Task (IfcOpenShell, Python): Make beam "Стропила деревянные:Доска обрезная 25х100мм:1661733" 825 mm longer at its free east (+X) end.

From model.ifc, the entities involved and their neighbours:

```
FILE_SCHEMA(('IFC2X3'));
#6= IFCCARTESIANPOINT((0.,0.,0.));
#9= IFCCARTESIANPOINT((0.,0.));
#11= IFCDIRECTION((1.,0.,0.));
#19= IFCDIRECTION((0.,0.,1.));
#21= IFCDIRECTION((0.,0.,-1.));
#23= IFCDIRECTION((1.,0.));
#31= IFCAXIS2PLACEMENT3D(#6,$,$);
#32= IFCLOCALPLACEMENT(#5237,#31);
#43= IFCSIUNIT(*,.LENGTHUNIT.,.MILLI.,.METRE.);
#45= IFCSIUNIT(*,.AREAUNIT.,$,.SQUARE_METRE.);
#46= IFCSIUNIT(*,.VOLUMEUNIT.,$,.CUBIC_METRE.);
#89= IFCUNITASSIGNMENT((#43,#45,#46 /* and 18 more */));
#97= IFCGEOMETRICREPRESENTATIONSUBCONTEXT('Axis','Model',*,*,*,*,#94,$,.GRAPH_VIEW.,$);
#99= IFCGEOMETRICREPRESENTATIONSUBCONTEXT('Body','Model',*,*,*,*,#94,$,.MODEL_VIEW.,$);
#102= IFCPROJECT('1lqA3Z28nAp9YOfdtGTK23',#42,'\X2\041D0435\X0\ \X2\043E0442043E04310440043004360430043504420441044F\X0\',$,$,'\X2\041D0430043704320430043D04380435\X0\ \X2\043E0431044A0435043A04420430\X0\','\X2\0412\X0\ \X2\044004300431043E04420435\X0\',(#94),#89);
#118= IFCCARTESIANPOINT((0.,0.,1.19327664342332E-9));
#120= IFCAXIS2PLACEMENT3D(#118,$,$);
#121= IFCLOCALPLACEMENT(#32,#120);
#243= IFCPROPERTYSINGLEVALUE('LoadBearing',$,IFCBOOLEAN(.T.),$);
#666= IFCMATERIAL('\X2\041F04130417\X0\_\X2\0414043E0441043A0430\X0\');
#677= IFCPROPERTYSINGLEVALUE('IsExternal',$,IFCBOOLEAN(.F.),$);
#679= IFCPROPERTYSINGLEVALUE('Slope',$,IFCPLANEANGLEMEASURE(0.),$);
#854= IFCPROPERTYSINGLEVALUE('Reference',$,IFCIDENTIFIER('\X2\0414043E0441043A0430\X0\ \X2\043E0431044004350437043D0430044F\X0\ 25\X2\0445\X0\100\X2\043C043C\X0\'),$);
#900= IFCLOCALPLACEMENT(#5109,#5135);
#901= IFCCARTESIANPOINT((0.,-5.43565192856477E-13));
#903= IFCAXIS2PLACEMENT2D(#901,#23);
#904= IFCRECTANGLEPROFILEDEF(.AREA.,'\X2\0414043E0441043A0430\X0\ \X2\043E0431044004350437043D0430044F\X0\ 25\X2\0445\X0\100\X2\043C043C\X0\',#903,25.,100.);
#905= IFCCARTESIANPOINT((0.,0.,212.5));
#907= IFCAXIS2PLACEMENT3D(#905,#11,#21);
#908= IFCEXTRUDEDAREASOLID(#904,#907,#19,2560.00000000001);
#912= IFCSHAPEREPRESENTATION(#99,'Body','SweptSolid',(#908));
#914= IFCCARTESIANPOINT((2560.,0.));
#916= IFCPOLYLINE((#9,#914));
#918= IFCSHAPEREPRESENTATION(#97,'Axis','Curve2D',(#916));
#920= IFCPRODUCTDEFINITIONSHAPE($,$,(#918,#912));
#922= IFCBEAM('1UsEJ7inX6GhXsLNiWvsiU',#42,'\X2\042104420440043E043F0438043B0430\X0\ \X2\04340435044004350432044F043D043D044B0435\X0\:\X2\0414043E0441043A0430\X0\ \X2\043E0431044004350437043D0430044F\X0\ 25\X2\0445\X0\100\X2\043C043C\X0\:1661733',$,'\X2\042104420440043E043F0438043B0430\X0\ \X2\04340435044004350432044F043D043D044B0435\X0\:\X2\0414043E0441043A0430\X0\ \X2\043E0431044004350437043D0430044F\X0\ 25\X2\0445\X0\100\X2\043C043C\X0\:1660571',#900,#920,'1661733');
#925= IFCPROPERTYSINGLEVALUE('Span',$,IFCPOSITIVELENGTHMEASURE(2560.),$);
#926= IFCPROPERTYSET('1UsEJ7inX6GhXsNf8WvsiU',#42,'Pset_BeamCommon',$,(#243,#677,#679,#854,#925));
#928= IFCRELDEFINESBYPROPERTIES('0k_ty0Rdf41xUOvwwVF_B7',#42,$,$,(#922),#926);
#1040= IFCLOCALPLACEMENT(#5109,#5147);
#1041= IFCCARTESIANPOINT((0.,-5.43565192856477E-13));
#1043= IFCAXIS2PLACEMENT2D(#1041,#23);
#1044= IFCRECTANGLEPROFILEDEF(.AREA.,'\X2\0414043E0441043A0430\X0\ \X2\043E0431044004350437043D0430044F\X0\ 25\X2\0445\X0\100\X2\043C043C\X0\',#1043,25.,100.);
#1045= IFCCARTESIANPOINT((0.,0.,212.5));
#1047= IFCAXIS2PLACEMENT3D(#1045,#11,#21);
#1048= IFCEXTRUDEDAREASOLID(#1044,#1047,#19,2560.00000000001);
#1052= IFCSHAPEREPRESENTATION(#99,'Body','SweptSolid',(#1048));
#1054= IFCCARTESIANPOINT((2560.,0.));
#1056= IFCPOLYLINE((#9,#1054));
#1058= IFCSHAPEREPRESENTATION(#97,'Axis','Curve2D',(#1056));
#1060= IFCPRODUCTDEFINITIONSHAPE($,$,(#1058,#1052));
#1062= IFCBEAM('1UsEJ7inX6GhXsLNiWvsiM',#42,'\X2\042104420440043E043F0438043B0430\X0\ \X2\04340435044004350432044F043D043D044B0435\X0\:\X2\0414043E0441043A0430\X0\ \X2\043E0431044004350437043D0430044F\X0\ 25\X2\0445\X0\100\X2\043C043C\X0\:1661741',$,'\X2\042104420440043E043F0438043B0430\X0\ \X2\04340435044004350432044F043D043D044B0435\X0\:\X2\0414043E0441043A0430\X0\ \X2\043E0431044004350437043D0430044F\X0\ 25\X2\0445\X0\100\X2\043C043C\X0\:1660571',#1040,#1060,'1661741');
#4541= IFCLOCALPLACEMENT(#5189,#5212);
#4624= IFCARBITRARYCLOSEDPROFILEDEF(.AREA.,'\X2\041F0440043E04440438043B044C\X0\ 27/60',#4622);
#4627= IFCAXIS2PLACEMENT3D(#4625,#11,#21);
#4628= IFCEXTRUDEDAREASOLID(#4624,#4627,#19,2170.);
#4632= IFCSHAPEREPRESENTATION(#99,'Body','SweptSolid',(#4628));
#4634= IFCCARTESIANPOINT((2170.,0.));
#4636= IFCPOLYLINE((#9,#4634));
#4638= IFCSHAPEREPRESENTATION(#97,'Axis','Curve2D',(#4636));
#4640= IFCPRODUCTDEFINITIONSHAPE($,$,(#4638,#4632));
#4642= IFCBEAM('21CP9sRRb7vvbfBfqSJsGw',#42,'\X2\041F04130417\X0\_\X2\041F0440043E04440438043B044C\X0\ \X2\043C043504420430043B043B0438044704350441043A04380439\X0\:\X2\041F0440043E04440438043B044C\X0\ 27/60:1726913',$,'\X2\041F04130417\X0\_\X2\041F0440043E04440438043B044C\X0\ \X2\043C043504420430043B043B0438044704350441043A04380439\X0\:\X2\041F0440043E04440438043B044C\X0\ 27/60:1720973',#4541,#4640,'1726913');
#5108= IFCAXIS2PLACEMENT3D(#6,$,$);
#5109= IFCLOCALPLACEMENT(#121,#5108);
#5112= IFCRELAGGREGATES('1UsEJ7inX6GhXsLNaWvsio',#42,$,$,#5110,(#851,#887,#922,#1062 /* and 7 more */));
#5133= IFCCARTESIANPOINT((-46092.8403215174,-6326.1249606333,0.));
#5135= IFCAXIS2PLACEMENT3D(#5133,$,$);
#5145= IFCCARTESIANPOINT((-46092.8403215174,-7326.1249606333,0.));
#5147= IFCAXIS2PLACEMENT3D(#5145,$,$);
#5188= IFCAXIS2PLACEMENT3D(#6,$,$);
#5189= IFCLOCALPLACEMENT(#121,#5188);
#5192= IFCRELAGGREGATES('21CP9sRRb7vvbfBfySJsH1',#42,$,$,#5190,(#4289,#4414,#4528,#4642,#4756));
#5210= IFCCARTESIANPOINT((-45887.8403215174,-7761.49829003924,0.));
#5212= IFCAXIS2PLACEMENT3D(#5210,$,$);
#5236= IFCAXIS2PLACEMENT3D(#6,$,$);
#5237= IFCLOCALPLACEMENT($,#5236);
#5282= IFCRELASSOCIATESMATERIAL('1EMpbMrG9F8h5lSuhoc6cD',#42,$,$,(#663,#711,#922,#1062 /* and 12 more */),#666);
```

```python
import numpy as np
import ifcopenshell
import ifcopenshell.api.pset
import ifcopenshell.util.element
import ifcopenshell.util.representation
import ifcopenshell.util.unit

model = ifcopenshell.open("model.ifc")
unit_scale = ifcopenshell.util.unit.calculate_unit_scale(model)

member = model.by_guid("1UsEJ7inX6GhXsLNiWvsiU")
change = 0.825 / unit_scale

# The extrusion runs towards the end named, so only its depth changes.
body = ifcopenshell.util.representation.get_representation(member, "Model", "Body")
solid = body.Items[0]
old_length = solid.Depth
solid.Depth += change

# Move the axis end point with it.
axis = next(r for r in member.Representation.Representations if r.RepresentationIdentifier == "Axis").Items[0]
start, end = (np.array(p.Coordinates) for p in axis.Points)
end = end + (end - start) / np.linalg.norm(end - start) * change
point = model.createIfcCartesianPoint(end.tolist())
axis.Points = [axis.Points[0], point]

# Update the stored length and volume.
pset = model.by_id(ifcopenshell.util.element.get_pset(member, "Pset_BeamCommon", should_inherit=False)["id"])
ifcopenshell.api.pset.edit_pset(model, pset=pset, properties={
    "Span": model.create_entity("IfcPositiveLengthMeasure", solid.Depth),
})

print(f"length {old_length:g} -> {solid.Depth:g}")

model.write("model_edited.ifc")
```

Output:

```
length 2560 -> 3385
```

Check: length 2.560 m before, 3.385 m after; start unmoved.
